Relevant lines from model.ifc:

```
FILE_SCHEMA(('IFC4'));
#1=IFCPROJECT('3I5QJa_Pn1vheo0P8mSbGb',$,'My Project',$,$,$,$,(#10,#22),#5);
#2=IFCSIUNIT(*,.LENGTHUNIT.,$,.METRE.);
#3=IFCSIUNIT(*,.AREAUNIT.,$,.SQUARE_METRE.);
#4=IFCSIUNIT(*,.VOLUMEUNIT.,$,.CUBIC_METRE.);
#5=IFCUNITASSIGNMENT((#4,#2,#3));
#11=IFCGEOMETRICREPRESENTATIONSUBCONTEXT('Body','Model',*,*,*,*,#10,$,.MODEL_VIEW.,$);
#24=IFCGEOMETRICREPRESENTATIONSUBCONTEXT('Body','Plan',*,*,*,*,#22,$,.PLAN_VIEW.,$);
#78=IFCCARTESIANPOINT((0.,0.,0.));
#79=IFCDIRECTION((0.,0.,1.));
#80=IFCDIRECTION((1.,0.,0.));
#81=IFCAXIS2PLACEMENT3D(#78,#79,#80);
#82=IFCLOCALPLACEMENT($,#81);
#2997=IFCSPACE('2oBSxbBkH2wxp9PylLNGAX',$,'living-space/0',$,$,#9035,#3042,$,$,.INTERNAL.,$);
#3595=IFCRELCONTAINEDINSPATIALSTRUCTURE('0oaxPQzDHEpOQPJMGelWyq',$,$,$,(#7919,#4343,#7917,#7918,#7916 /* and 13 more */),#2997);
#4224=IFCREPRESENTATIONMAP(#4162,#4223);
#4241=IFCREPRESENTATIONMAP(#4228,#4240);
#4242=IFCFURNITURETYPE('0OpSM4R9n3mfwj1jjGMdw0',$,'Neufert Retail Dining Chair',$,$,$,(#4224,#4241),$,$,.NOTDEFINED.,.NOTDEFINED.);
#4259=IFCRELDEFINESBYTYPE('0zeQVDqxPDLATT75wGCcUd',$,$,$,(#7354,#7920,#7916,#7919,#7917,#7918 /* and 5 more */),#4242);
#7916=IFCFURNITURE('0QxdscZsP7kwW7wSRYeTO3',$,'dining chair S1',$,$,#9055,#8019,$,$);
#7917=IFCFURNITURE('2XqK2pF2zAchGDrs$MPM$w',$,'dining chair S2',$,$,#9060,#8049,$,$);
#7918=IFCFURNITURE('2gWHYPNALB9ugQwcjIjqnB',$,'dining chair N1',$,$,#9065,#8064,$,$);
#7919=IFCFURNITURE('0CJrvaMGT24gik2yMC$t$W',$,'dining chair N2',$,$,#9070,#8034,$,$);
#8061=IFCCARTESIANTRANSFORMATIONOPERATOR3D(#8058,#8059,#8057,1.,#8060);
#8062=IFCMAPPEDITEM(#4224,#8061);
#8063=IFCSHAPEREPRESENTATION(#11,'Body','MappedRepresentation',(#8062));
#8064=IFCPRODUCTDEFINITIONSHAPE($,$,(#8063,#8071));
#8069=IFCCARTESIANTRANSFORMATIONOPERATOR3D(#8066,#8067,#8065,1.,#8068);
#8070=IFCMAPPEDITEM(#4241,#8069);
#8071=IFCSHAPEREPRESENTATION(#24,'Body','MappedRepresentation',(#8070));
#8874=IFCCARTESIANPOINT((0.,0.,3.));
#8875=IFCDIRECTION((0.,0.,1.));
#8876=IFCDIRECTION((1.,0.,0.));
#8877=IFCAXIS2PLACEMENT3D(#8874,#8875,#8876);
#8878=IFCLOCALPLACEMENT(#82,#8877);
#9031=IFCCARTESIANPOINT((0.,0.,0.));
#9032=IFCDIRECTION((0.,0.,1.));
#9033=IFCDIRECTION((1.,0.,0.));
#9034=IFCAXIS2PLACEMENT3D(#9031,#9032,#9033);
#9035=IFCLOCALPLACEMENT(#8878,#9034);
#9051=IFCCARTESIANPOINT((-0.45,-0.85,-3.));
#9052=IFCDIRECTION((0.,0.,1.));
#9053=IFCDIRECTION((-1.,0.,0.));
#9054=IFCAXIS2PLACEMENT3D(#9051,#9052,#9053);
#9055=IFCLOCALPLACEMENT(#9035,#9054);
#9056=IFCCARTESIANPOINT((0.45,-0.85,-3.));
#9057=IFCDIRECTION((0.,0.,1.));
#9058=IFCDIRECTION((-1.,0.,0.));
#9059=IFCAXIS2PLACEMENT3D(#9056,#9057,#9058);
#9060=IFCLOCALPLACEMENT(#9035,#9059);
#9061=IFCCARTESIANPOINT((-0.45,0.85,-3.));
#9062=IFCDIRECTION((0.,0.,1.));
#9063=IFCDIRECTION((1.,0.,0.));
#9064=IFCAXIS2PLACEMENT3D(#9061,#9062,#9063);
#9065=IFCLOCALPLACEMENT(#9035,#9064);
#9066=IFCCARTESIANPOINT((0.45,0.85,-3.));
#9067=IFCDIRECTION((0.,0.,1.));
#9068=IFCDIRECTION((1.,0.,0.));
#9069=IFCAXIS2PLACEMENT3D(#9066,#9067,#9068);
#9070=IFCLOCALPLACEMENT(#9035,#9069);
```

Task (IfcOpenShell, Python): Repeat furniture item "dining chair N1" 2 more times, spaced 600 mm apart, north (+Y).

```python
import numpy as np
import ifcopenshell
import ifcopenshell.api.geometry
import ifcopenshell.api.root
import ifcopenshell.util.element
import ifcopenshell.util.placement

model = ifcopenshell.open("model.ifc")

source = model.by_id(7918)
base = ifcopenshell.util.placement.get_local_placement(source.ObjectPlacement)
step = np.array([0.0, 1.0, 0.0]) * 0.6

for i in range(1, 3):
    copy = ifcopenshell.api.root.copy_class(model, product=source)
    copy.Representation = ifcopenshell.util.element.copy_deep(
        model, source.Representation, exclude=["IfcGeometricRepresentationContext", "IfcRepresentationMap"]
    )
    matrix = base.copy()
    matrix[:3, 3] += i * step
    print("added at", matrix[:3, 3].round(3) + 0.0)
    ifcopenshell.api.geometry.edit_object_placement(model, product=copy, matrix=matrix, is_si=False)

model.write("model-out.ifc")
```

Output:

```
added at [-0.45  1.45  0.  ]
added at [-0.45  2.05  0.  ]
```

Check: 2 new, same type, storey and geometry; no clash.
